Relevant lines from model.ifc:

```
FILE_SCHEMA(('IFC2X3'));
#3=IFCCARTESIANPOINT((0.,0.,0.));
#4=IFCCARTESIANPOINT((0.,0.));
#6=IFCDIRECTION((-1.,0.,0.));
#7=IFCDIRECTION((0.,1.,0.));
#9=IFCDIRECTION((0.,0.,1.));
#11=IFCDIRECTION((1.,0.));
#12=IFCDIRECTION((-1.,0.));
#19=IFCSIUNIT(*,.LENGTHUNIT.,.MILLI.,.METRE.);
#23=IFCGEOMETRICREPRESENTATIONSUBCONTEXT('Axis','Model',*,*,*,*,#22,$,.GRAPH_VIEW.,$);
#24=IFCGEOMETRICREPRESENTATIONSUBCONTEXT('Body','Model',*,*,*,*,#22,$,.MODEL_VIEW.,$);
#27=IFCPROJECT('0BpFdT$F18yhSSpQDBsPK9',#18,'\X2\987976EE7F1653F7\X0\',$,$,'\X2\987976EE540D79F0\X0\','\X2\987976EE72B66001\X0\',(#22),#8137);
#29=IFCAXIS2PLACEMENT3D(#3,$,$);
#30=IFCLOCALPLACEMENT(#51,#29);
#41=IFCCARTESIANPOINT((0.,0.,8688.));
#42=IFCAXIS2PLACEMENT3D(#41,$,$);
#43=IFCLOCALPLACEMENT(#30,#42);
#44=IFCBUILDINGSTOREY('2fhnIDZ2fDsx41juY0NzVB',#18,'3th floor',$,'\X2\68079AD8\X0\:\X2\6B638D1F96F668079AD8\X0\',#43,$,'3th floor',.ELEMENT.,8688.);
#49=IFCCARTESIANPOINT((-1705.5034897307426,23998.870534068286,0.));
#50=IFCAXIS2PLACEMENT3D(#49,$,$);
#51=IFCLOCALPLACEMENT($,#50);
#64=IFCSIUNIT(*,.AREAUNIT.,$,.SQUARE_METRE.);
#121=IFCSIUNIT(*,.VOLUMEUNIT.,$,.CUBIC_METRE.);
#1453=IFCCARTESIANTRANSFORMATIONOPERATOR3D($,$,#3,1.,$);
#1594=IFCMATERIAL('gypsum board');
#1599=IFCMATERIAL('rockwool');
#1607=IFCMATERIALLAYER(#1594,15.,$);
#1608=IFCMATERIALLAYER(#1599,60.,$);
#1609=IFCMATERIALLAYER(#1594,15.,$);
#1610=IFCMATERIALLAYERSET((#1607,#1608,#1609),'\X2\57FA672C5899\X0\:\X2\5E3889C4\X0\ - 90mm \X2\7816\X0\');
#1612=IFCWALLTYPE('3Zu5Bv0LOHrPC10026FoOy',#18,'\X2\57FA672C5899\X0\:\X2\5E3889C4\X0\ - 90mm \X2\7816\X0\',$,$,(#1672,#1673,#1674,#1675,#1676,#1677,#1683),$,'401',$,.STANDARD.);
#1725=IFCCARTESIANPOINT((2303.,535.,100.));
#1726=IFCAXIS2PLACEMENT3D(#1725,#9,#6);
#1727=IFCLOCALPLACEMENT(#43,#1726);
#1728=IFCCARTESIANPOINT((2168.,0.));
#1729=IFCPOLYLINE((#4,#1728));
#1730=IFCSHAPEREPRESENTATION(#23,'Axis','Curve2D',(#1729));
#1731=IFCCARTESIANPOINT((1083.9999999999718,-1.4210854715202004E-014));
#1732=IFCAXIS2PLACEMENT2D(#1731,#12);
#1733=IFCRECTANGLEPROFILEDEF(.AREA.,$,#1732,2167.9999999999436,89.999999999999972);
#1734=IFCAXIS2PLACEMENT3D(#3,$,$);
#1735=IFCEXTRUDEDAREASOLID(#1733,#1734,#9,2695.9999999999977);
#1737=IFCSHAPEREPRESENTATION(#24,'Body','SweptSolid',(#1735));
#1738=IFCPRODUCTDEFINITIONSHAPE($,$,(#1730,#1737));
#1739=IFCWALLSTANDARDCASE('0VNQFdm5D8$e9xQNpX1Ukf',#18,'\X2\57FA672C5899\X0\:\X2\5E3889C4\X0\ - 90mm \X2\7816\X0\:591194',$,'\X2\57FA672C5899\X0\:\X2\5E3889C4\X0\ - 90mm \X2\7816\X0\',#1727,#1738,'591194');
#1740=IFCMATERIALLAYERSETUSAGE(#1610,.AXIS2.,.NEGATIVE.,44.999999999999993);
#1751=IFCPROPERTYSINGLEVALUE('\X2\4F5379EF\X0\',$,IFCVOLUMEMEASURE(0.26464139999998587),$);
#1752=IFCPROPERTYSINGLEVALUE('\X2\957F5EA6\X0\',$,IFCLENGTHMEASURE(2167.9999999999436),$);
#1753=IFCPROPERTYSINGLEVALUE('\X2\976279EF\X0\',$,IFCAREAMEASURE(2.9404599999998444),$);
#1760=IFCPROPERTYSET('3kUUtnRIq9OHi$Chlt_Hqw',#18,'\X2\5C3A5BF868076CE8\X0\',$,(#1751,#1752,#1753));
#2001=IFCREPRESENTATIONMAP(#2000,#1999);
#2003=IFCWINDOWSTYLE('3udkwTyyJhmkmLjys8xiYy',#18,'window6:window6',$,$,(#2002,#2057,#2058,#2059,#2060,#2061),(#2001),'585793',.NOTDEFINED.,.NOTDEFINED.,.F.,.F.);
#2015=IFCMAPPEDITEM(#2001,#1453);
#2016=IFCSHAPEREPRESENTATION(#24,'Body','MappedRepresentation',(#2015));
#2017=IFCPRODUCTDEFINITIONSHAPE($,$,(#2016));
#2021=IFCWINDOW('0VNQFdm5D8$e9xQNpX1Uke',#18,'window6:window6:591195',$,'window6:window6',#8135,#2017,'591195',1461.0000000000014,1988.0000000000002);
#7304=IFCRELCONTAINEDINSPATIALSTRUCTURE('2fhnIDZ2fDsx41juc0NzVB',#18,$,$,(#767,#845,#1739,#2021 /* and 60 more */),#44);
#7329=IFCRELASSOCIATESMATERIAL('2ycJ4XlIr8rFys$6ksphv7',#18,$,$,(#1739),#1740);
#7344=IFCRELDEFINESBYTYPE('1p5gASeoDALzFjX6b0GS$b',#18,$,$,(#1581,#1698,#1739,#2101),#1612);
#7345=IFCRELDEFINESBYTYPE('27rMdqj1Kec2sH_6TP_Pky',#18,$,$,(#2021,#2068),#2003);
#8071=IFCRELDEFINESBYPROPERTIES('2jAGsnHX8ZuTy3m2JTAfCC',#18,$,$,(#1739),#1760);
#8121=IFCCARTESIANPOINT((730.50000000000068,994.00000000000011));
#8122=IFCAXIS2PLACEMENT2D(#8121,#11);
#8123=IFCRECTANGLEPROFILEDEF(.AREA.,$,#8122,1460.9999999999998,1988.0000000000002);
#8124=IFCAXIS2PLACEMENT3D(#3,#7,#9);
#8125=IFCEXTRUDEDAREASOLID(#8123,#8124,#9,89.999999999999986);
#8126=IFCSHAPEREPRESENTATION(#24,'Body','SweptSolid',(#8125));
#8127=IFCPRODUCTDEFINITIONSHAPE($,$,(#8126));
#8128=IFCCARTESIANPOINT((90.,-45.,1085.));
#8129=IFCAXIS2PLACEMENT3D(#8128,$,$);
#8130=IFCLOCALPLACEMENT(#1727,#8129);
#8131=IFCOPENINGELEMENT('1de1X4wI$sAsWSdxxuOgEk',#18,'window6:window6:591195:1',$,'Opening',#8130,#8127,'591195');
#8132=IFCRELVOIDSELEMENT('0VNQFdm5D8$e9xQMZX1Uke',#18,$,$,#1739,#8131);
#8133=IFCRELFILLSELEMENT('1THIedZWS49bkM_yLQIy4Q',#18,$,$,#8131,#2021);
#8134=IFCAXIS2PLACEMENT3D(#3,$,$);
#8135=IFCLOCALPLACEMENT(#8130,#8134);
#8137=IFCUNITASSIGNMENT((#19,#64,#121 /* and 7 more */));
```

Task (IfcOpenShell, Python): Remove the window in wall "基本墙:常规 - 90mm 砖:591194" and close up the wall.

```python
import ifcopenshell
import ifcopenshell.api.feature
import ifcopenshell.api.pset
import ifcopenshell.api.root
import ifcopenshell.geom
import ifcopenshell.util.element
import ifcopenshell.util.shape
import ifcopenshell.util.unit

model = ifcopenshell.open("model.ifc")
area_scale = ifcopenshell.util.unit.calculate_unit_scale(model, "AREAUNIT")
volume_scale = ifcopenshell.util.unit.calculate_unit_scale(model, "VOLUMEUNIT")
settings = ifcopenshell.geom.settings()


def volume(element):
    """Net volume in cubic metres, openings subtracted."""
    shape = ifcopenshell.geom.create_shape(settings, element)
    return ifcopenshell.util.shape.get_volume(shape.geometry)


window = model.by_guid("0VNQFdm5D8$e9xQNpX1Uke")
opening = window.FillsVoids[0].RelatingOpeningElement
wall = opening.VoidsElements[0].RelatingBuildingElement
before = volume(wall)

ifcopenshell.api.root.remove_product(model, product=window)
ifcopenshell.api.feature.remove_feature(model, feature=opening)

after = volume(wall)
thickness = 0.09  # wall thickness in metres

# Update the wall's stored quantities.
pset = model.by_id(ifcopenshell.util.element.get_pset(wall, "尺寸标注", should_inherit=False)["id"])
ifcopenshell.api.pset.edit_pset(model, pset=pset, properties={
    "体积": model.create_entity("IfcVolumeMeasure", after / volume_scale),
    "面积": model.create_entity("IfcAreaMeasure", after / thickness / area_scale),
})

print(f"wall volume {before:.3f} -> {after:.3f} m3")

model.write("model_v2.ifc")
```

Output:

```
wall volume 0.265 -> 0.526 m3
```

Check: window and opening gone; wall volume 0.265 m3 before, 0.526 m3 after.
